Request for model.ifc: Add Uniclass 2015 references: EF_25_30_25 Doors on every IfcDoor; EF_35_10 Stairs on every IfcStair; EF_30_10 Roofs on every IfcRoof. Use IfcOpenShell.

First a look at what the model holds.

```python
import ifcopenshell

model = ifcopenshell.open("model.ifc")
print(model.schema)
print("classifications:", [c.Name for c in model.by_type("IfcClassification")])
for ifc_class in ("IfcDoor", "IfcRoof", "IfcStair", "IfcWall", "IfcWindow"):
    print(ifc_class, len(model.by_type(ifc_class)))
```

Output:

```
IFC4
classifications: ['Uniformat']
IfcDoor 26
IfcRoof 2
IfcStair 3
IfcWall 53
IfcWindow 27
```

```python
import ifcopenshell
import ifcopenshell.api.classification

model = ifcopenshell.open("model.ifc")

system = ifcopenshell.api.classification.add_classification(model, classification="Uniclass 2015")

codes = {
    "IfcDoor": ("EF_25_30_25", "Doors"),
    "IfcStair": ("EF_35_10", "Stairs"),
    "IfcRoof": ("EF_30_10", "Roofs"),
}
for ifc_class, (code, name) in codes.items():
    products = model.by_type(ifc_class)
    ifcopenshell.api.classification.add_reference(
        model, products=products, classification=system, identification=code, name=name
    )
    print(code, len(products))

model.write("model_edited.ifc")
```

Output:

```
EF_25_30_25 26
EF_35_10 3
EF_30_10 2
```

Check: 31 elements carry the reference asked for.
